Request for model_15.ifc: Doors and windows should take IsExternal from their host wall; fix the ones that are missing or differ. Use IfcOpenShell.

First a look at what the model holds.

```python
import ifcopenshell
import ifcopenshell.util.element

model = ifcopenshell.open("model_15.ifc")
print(model.schema)
seen = {}
for e in model.by_type("IfcDoor") + model.by_type("IfcWindow"):
    if not e.FillsVoids:
        continue
    host = e.FillsVoids[0].RelatingOpeningElement.VoidsElements[0].RelatingBuildingElement
    own = ifcopenshell.util.element.get_pset(e, f"Pset_{e.is_a()[3:].removesuffix('StandardCase')}Common", "IsExternal")
    wall = ifcopenshell.util.element.get_pset(host, "Pset_WallCommon", "IsExternal")
    seen[e.is_a(), own, wall] = seen.get((e.is_a(), own, wall), 0) + 1
for (cls, own, wall), count in sorted(seen.items(), key=str):
    print(count, cls, "IsExternal:", own, "| host wall:", wall)
```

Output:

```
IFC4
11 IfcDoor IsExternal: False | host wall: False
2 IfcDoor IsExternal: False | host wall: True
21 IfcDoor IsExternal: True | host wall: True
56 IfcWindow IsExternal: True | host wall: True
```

```python
import ifcopenshell
import ifcopenshell.api.pset
import ifcopenshell.util.element

model = ifcopenshell.open("model_15.ifc")

count = 0
for ifc_class, pset_name in (("IfcDoor", "Pset_DoorCommon"), ("IfcWindow", "Pset_WindowCommon")):
    for e in model.by_type(ifc_class):
        if not e.FillsVoids:
            continue
        host = e.FillsVoids[0].RelatingOpeningElement.VoidsElements[0].RelatingBuildingElement
        external = ifcopenshell.util.element.get_pset(host, "Pset_WallCommon", "IsExternal")
        if external is None or ifcopenshell.util.element.get_pset(e, pset_name, "IsExternal") == external:
            continue
        pset = ifcopenshell.api.pset.add_pset(model, product=e, name=pset_name)
        ifcopenshell.api.pset.edit_pset(model, pset=pset, properties={"IsExternal": external})
        count += 1

print(count, "updated")

model.write("model_15_v2.ifc")
```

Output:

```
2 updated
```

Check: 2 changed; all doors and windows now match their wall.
